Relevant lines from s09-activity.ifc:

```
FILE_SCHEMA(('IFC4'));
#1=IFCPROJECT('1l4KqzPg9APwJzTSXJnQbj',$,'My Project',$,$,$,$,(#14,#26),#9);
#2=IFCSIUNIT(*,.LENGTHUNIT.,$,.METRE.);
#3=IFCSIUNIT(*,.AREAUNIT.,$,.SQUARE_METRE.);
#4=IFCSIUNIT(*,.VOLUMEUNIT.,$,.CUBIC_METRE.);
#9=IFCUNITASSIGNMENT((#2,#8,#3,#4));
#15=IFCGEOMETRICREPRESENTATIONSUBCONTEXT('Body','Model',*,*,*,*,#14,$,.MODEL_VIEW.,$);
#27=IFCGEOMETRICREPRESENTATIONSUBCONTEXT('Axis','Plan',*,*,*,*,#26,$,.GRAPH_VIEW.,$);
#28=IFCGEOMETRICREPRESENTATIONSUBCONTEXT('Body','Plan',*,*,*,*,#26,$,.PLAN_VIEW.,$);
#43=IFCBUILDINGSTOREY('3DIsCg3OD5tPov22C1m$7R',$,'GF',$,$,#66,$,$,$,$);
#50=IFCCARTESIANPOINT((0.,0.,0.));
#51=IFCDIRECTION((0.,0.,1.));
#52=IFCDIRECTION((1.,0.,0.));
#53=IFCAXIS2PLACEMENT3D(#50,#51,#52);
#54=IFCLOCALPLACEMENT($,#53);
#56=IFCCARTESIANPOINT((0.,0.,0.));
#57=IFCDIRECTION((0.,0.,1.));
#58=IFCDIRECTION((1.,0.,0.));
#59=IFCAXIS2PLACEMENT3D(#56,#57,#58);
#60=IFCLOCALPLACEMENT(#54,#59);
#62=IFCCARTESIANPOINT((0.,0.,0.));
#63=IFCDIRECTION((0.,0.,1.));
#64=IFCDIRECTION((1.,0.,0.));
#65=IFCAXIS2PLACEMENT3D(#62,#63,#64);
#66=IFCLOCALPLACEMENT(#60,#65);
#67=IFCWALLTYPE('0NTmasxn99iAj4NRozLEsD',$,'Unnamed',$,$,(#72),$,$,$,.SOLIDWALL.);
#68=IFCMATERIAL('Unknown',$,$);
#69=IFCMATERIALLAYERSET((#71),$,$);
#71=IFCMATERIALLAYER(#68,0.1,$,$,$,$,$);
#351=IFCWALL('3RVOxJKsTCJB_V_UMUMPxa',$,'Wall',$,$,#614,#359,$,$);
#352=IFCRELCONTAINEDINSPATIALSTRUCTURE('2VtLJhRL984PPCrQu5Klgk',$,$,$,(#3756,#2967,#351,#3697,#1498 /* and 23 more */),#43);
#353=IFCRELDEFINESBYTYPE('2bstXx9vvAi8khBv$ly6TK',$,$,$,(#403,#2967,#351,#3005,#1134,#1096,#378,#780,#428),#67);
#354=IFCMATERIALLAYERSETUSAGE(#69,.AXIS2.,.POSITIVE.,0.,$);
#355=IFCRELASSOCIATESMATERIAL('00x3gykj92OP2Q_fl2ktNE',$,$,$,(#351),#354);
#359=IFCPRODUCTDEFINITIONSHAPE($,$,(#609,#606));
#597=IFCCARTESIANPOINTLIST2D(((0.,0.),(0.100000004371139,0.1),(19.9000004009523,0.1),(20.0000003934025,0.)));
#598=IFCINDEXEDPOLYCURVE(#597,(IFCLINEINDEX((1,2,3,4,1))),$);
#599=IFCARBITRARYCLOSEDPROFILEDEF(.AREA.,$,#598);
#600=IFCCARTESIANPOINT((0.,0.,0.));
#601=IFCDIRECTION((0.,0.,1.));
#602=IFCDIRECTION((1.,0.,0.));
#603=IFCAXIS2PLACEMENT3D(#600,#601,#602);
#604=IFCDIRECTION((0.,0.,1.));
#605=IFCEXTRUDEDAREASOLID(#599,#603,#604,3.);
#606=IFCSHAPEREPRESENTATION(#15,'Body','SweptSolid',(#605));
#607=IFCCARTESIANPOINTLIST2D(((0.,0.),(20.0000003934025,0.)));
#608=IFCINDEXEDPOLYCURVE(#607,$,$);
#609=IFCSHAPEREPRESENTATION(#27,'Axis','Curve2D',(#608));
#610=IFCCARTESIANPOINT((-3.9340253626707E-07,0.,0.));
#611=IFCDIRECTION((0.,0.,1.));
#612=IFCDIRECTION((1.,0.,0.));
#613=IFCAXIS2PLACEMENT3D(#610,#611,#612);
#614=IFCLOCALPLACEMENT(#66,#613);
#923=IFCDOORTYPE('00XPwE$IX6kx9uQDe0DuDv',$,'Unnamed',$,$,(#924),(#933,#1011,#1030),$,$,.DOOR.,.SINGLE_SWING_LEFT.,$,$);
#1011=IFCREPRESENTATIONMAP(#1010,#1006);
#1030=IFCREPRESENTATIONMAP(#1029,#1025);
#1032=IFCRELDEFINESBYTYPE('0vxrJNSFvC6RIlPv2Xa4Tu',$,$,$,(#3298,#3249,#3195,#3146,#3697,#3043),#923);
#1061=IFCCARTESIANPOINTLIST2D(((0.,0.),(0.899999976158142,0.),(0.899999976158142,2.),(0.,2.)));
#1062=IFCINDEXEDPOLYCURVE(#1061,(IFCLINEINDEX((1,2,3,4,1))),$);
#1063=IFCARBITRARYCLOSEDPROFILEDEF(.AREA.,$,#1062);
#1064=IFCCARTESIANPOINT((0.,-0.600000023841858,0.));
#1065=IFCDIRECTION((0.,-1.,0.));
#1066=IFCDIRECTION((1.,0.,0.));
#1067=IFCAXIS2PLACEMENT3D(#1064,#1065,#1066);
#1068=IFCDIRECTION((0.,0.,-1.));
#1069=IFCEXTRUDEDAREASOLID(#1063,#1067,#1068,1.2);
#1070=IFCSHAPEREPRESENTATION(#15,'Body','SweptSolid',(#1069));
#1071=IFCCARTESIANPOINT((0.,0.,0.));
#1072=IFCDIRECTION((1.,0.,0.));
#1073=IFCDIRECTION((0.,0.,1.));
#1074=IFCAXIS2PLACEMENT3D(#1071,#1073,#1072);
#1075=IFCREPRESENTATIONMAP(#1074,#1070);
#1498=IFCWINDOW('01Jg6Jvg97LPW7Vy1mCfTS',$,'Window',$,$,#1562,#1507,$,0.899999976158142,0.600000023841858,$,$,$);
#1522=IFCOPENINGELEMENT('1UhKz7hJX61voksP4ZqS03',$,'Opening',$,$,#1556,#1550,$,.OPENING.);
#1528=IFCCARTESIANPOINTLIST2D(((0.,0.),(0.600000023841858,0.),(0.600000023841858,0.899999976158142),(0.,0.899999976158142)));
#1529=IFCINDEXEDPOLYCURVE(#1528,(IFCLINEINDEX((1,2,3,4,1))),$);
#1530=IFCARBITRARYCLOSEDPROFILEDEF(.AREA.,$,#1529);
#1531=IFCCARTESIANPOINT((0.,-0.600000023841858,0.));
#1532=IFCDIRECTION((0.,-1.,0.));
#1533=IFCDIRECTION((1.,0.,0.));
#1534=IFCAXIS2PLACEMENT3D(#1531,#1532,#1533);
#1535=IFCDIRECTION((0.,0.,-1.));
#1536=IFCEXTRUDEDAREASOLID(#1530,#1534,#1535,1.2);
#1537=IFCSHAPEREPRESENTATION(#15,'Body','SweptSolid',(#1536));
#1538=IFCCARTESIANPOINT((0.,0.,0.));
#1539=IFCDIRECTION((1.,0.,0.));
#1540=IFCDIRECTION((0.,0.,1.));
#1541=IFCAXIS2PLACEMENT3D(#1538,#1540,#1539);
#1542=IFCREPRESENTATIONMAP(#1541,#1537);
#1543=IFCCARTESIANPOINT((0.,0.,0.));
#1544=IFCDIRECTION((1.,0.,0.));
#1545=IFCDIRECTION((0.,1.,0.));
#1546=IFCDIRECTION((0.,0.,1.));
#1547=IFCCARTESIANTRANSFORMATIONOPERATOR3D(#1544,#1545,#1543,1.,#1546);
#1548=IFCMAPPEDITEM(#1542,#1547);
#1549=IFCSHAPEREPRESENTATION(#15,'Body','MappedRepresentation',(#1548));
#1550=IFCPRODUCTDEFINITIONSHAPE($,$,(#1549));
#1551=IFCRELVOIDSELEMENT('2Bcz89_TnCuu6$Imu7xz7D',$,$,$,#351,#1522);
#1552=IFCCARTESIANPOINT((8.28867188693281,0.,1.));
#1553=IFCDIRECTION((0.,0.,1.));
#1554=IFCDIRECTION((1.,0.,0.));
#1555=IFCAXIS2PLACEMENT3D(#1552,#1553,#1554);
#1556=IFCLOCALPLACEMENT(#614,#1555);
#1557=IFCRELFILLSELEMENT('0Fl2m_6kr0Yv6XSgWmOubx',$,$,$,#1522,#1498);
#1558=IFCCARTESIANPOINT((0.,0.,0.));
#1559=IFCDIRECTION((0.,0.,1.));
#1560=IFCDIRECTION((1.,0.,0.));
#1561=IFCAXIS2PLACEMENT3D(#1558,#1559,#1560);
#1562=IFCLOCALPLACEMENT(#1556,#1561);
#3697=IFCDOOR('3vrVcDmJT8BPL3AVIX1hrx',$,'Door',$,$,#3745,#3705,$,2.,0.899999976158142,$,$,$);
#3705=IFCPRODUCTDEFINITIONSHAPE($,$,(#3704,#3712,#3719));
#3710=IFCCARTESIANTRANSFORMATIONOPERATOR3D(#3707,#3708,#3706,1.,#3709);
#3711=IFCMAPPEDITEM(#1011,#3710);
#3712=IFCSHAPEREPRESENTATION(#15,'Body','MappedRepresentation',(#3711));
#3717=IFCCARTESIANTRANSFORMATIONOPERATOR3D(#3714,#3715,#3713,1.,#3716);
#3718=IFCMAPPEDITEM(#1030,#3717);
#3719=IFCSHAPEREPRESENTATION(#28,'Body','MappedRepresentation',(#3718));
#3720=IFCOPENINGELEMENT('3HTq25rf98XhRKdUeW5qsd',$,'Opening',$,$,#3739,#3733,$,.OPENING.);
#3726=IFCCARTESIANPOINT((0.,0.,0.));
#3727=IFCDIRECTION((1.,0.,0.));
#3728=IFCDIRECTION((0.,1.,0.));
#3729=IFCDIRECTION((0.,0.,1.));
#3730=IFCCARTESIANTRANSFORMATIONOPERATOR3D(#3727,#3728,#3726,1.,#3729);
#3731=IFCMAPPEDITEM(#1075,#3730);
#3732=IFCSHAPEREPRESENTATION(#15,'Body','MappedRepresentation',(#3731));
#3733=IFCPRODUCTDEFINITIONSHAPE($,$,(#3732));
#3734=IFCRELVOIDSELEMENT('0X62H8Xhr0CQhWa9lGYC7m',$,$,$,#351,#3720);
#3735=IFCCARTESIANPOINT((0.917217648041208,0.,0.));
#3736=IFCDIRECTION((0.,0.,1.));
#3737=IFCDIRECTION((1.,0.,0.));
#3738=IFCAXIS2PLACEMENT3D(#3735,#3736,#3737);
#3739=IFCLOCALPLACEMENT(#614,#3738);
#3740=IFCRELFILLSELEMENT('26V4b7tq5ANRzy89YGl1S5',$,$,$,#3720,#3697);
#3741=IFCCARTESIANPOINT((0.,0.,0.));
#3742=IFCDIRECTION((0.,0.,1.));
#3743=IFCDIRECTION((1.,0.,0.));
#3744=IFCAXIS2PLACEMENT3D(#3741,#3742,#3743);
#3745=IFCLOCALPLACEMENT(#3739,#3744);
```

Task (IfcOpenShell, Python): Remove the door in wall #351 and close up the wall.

```python
import ifcopenshell
import ifcopenshell.api.feature
import ifcopenshell.api.root
import ifcopenshell.geom
import ifcopenshell.util.shape

model = ifcopenshell.open("s09-activity.ifc")
settings = ifcopenshell.geom.settings()


def volume(element):
    """Net volume in cubic metres, openings subtracted."""
    shape = ifcopenshell.geom.create_shape(settings, element)
    return ifcopenshell.util.shape.get_volume(shape.geometry)


door = model.by_guid("3vrVcDmJT8BPL3AVIX1hrx")
opening = door.FillsVoids[0].RelatingOpeningElement
wall = opening.VoidsElements[0].RelatingBuildingElement
before = volume(wall)

ifcopenshell.api.root.remove_product(model, product=door)
ifcopenshell.api.feature.remove_feature(model, feature=opening)

after = volume(wall)

print(f"wall volume {before:.3f} -> {after:.3f} m3")

model.write("s09-activity-out.ifc")
```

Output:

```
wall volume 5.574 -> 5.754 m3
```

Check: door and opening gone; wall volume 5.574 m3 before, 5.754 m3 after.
